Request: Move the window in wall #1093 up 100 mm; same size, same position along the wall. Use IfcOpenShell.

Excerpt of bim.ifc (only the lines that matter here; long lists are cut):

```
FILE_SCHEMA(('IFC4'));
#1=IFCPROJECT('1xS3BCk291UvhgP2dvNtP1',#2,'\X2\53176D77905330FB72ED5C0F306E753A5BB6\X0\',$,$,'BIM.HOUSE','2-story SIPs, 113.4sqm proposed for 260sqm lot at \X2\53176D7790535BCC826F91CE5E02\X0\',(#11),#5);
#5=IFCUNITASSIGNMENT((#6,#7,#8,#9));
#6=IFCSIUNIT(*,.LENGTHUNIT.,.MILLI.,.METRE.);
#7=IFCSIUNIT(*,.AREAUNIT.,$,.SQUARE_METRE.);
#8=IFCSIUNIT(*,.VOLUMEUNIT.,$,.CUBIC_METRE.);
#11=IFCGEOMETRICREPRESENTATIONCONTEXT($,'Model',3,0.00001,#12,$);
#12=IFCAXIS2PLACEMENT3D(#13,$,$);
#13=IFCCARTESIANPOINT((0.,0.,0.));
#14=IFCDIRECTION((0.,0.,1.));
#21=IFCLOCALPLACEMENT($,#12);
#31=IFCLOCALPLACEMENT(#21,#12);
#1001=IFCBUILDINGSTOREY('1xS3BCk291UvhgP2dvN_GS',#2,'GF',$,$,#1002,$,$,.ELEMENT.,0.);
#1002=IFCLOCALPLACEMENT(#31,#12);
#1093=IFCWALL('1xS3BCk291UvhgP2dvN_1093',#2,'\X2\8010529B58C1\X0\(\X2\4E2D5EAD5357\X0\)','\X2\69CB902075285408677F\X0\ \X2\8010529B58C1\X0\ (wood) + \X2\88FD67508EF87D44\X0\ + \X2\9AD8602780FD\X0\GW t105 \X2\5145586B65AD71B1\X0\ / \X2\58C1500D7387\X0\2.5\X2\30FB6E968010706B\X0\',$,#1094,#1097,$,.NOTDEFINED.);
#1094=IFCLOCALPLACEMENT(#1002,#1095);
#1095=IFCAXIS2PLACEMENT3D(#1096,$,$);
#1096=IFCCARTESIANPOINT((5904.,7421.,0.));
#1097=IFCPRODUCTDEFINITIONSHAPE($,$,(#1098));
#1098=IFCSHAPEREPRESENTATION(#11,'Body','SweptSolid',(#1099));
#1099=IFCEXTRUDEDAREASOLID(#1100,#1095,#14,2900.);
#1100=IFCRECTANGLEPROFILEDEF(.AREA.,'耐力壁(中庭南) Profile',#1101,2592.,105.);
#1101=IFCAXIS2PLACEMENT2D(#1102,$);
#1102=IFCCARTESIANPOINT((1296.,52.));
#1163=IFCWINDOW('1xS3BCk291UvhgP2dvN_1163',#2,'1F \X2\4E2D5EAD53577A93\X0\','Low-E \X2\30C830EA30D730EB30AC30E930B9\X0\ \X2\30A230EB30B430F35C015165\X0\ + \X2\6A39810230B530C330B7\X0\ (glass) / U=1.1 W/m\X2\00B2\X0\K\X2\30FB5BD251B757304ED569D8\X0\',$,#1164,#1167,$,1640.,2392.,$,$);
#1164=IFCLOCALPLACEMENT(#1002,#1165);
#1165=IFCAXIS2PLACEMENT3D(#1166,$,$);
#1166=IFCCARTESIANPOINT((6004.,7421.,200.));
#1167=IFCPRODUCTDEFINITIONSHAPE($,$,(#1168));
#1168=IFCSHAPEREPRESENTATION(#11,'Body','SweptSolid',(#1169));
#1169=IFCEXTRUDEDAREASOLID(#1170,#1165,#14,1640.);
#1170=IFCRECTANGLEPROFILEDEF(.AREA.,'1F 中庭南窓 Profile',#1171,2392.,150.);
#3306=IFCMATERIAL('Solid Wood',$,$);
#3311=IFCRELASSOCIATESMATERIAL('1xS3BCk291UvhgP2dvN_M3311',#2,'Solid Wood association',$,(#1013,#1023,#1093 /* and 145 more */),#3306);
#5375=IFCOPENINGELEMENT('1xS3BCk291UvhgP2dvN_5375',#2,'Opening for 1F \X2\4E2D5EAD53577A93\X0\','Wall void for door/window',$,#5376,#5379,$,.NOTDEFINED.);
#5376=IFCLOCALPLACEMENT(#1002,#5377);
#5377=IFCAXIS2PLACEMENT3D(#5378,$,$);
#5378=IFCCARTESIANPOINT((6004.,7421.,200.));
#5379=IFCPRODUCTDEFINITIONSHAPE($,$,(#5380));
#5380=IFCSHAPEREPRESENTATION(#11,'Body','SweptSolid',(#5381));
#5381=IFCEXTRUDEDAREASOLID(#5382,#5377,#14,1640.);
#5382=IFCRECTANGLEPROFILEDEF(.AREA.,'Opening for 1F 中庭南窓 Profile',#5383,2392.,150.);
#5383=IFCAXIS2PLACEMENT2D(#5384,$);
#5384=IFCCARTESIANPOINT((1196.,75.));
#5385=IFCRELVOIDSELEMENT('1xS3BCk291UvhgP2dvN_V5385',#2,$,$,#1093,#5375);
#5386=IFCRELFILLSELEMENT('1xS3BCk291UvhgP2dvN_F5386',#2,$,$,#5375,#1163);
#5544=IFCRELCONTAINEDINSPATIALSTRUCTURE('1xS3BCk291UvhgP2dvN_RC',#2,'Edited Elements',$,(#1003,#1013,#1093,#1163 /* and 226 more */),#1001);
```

```python
import numpy as np
import ifcopenshell
import ifcopenshell.api.geometry
import ifcopenshell.util.placement
import ifcopenshell.util.unit

model = ifcopenshell.open("bim.ifc")
unit_scale = ifcopenshell.util.unit.calculate_unit_scale(model)

window = model.by_guid("1xS3BCk291UvhgP2dvN_1163")
opening = window.FillsVoids[0].RelatingOpeningElement
dz = 100.0

shift = np.array([0.0, 0.0, dz])
# The window is not placed relative to its opening, so move both.
for product in (opening, window):
    matrix = ifcopenshell.util.placement.get_local_placement(product.ObjectPlacement)
    matrix[:3, 3] += shift
    ifcopenshell.api.geometry.edit_object_placement(model, product=product, matrix=matrix, is_si=False)

print(f"moved by {dz * unit_scale:+.3f} m")

model.write("bim-out.ifc")
```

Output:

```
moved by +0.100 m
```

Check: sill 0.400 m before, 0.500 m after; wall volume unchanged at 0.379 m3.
